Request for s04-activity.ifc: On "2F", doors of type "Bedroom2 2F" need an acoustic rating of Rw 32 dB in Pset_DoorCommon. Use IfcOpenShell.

First a look at what the model holds.

```python
import ifcopenshell
import ifcopenshell.util.element

model = ifcopenshell.open("s04-activity.ifc")
print(model.schema)
storey = next(s for s in model.by_type("IfcBuildingStorey") if s.Name == "2F")
doors = [e for e in ifcopenshell.util.element.get_decomposition(storey) if e.is_a("IfcDoor")]
seen = {}
for e in doors:
    element_type = ifcopenshell.util.element.get_type(e)
    key = (element_type.Name if element_type != e and element_type else None, ifcopenshell.util.element.get_pset(e, "Pset_DoorCommon", "AcousticRating"))
    seen[key] = seen.get(key, 0) + 1
for (name, value), count in sorted(seen.items(), key=str):
    print(count, "x", name, "|", value)
```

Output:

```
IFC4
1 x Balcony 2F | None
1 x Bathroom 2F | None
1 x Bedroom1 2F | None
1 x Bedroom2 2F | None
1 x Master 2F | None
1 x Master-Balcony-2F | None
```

```python
import ifcopenshell
import ifcopenshell.api.pset
import ifcopenshell.util.element

model = ifcopenshell.open("s04-activity.ifc")

storey = next(s for s in model.by_type("IfcBuildingStorey") if s.Name == "2F")
doors = [e for e in ifcopenshell.util.element.get_decomposition(storey) if e.is_a("IfcDoor")]

count = 0
for e in doors:
    element_type = ifcopenshell.util.element.get_type(e)
    if element_type in (None, e) or element_type.Name != "Bedroom2 2F":
        continue
    # add_pset returns the element's existing set when there is one.
    pset = ifcopenshell.api.pset.add_pset(model, product=e, name="Pset_DoorCommon")
    ifcopenshell.api.pset.edit_pset(model, pset=pset, properties={"AcousticRating": "Rw 32 dB"})
    count += 1

print(count, "doors updated")

model.write("s04-activity_edited.ifc")
```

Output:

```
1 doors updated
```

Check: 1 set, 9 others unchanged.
